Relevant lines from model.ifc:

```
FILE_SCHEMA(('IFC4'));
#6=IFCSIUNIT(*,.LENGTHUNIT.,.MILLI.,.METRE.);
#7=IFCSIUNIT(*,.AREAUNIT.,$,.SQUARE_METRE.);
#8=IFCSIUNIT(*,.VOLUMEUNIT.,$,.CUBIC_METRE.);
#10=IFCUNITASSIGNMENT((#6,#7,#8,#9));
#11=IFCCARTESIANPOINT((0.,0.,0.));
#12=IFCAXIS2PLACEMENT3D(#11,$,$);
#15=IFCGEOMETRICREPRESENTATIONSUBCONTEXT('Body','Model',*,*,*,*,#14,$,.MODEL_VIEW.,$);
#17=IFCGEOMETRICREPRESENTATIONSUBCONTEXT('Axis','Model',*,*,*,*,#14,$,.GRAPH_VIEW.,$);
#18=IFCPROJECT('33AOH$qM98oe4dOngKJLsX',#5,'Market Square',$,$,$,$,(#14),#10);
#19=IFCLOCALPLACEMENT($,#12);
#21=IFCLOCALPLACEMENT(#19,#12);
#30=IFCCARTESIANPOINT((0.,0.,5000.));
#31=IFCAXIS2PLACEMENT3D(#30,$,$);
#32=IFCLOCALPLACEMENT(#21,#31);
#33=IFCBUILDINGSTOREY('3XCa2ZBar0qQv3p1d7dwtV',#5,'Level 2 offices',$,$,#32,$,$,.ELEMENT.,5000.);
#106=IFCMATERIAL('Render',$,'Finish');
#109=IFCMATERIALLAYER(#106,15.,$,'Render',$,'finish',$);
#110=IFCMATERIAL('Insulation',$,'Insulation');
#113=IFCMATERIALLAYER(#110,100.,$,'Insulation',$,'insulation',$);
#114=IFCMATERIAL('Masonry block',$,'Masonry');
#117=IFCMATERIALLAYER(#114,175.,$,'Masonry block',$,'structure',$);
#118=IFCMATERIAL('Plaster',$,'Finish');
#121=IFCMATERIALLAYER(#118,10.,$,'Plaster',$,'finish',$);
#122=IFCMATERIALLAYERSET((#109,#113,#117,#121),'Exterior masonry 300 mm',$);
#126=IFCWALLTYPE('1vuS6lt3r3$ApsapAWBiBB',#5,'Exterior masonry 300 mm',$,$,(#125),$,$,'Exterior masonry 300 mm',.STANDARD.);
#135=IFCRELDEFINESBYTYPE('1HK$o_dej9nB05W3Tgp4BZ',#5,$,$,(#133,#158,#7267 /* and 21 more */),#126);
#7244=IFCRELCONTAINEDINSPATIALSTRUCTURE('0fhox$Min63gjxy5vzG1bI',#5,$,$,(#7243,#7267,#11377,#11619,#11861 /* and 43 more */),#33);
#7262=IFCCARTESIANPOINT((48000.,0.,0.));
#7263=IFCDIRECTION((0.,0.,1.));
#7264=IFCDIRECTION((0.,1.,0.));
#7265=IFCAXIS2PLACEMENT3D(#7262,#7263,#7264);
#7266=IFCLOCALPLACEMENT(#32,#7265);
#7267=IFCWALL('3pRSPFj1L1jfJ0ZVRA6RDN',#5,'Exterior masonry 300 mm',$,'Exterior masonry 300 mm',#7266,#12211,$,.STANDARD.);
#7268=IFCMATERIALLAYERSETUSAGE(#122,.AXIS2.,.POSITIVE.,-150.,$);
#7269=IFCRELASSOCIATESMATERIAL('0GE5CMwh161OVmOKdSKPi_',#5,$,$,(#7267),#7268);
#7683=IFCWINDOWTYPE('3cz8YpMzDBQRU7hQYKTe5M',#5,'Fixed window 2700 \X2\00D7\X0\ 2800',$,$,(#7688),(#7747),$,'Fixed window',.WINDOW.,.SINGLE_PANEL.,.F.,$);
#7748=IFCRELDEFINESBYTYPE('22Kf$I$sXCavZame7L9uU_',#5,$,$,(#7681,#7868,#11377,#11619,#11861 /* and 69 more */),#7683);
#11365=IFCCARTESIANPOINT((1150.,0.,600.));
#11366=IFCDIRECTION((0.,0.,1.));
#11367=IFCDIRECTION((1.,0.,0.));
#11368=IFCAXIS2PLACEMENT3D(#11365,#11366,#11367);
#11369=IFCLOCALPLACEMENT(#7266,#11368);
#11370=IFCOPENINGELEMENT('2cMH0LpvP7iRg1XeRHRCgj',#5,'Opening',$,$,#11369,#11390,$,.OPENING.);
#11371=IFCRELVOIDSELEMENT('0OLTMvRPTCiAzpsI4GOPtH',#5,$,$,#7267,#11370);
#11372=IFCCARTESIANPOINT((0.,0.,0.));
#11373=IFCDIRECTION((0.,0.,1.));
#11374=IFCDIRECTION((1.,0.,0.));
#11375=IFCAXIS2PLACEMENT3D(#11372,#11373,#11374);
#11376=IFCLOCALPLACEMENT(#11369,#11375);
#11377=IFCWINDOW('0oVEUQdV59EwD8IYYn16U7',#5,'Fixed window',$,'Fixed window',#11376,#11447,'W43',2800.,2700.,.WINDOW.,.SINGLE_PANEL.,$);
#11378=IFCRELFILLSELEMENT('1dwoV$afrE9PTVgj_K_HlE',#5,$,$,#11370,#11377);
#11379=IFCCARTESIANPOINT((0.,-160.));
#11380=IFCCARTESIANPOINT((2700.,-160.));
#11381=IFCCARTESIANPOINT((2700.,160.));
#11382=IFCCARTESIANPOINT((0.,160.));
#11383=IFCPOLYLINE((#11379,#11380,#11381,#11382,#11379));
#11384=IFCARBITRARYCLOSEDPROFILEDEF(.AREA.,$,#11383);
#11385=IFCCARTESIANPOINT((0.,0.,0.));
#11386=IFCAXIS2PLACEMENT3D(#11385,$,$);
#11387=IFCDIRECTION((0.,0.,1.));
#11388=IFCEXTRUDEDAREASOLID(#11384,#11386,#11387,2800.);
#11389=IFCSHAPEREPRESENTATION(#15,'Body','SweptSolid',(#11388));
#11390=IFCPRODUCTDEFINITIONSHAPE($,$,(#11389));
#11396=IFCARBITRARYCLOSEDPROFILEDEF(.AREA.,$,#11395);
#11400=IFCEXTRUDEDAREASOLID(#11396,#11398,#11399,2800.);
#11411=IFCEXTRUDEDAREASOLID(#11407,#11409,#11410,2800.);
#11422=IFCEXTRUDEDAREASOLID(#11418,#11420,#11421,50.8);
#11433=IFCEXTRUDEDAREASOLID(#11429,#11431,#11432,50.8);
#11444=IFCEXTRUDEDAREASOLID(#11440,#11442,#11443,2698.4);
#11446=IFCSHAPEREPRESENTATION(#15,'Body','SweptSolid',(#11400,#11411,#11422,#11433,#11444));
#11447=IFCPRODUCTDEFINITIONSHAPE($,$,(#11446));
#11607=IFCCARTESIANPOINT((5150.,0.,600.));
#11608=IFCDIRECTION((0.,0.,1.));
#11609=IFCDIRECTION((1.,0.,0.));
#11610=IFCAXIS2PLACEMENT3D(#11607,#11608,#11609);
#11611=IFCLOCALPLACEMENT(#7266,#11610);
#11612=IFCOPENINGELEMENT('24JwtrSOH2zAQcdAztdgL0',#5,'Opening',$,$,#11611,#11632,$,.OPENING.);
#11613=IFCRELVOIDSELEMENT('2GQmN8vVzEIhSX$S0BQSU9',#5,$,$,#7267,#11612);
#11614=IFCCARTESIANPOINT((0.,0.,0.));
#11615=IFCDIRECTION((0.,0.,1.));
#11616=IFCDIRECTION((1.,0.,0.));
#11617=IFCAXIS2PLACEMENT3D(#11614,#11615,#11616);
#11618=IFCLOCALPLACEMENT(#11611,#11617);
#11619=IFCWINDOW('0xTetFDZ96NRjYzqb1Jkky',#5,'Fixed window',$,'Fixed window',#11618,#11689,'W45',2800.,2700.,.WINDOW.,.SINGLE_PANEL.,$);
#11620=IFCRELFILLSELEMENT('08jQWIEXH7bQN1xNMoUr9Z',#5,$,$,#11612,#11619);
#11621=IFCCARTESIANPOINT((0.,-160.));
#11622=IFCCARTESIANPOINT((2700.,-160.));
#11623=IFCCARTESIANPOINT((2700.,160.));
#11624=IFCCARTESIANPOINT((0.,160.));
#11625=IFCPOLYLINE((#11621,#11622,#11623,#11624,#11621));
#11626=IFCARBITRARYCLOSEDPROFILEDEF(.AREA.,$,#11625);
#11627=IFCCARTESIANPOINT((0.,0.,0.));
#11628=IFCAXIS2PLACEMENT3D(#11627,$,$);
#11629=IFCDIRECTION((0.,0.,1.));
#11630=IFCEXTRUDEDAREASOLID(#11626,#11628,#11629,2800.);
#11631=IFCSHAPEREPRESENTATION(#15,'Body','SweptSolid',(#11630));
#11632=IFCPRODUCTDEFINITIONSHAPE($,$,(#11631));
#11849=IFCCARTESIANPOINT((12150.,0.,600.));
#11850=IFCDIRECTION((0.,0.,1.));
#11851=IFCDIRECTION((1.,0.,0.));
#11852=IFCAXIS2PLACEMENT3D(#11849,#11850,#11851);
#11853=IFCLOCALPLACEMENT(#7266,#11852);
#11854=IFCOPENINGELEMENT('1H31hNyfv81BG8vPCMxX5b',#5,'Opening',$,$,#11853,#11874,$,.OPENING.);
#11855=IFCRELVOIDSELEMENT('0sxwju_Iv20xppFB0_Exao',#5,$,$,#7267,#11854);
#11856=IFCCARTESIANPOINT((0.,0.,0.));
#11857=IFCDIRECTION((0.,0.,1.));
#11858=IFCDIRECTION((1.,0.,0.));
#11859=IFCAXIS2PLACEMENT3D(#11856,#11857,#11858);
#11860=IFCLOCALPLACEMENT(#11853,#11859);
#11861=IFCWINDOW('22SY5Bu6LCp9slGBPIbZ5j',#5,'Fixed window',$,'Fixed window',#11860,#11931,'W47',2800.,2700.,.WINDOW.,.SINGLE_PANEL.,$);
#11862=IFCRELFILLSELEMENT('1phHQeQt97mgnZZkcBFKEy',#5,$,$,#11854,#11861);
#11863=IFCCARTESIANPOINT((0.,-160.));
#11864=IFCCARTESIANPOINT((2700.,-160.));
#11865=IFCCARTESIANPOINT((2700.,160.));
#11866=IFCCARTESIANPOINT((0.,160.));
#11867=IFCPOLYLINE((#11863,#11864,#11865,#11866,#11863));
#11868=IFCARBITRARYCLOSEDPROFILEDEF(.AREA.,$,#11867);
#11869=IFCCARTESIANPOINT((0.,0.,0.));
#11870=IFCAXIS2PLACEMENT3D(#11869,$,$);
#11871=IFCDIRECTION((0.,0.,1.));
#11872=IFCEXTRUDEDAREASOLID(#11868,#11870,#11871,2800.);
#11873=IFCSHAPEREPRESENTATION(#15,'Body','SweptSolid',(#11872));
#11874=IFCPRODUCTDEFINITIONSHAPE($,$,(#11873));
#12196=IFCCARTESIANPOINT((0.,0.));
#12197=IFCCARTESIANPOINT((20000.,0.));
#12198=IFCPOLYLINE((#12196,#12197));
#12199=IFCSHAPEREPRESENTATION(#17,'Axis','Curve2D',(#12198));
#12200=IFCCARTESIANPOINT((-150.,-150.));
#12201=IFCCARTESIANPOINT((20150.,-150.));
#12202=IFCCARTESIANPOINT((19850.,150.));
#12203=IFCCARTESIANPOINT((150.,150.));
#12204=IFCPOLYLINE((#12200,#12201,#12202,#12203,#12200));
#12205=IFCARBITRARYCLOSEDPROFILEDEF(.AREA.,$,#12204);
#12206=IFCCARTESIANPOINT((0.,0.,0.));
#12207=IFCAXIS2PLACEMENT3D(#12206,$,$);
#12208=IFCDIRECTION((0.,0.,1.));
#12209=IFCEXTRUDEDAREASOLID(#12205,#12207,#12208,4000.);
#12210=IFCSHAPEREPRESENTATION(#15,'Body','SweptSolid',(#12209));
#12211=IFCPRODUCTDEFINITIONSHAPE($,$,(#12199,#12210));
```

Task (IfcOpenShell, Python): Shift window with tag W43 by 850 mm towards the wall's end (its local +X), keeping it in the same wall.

```python
import ifcopenshell
import ifcopenshell.api.geometry
import ifcopenshell.util.placement
import ifcopenshell.util.unit

model = ifcopenshell.open("model.ifc")
unit_scale = ifcopenshell.util.unit.calculate_unit_scale(model)

window = model.by_guid("0oVEUQdV59EwD8IYYn16U7")
opening = window.FillsVoids[0].RelatingOpeningElement
wall = opening.VoidsElements[0].RelatingBuildingElement

wall_matrix = ifcopenshell.util.placement.get_local_placement(wall.ObjectPlacement)
shift = wall_matrix[:3, 0] * 0.85 / unit_scale
before = ifcopenshell.util.placement.get_local_placement(window.ObjectPlacement)[:3, 3].copy()

# The window is placed relative to its opening, so it follows when the opening moves.
matrix = ifcopenshell.util.placement.get_local_placement(opening.ObjectPlacement)
matrix[:3, 3] += shift
ifcopenshell.api.geometry.edit_object_placement(
    model, product=opening, matrix=matrix, is_si=False, should_transform_children=True
)

after = ifcopenshell.util.placement.get_local_placement(window.ObjectPlacement)[:3, 3]
print("window moved by", (after - before).round(3) + 0.0)

model.write("model_rev.ifc")
```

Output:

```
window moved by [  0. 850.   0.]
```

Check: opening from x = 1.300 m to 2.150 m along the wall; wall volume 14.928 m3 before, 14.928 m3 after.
